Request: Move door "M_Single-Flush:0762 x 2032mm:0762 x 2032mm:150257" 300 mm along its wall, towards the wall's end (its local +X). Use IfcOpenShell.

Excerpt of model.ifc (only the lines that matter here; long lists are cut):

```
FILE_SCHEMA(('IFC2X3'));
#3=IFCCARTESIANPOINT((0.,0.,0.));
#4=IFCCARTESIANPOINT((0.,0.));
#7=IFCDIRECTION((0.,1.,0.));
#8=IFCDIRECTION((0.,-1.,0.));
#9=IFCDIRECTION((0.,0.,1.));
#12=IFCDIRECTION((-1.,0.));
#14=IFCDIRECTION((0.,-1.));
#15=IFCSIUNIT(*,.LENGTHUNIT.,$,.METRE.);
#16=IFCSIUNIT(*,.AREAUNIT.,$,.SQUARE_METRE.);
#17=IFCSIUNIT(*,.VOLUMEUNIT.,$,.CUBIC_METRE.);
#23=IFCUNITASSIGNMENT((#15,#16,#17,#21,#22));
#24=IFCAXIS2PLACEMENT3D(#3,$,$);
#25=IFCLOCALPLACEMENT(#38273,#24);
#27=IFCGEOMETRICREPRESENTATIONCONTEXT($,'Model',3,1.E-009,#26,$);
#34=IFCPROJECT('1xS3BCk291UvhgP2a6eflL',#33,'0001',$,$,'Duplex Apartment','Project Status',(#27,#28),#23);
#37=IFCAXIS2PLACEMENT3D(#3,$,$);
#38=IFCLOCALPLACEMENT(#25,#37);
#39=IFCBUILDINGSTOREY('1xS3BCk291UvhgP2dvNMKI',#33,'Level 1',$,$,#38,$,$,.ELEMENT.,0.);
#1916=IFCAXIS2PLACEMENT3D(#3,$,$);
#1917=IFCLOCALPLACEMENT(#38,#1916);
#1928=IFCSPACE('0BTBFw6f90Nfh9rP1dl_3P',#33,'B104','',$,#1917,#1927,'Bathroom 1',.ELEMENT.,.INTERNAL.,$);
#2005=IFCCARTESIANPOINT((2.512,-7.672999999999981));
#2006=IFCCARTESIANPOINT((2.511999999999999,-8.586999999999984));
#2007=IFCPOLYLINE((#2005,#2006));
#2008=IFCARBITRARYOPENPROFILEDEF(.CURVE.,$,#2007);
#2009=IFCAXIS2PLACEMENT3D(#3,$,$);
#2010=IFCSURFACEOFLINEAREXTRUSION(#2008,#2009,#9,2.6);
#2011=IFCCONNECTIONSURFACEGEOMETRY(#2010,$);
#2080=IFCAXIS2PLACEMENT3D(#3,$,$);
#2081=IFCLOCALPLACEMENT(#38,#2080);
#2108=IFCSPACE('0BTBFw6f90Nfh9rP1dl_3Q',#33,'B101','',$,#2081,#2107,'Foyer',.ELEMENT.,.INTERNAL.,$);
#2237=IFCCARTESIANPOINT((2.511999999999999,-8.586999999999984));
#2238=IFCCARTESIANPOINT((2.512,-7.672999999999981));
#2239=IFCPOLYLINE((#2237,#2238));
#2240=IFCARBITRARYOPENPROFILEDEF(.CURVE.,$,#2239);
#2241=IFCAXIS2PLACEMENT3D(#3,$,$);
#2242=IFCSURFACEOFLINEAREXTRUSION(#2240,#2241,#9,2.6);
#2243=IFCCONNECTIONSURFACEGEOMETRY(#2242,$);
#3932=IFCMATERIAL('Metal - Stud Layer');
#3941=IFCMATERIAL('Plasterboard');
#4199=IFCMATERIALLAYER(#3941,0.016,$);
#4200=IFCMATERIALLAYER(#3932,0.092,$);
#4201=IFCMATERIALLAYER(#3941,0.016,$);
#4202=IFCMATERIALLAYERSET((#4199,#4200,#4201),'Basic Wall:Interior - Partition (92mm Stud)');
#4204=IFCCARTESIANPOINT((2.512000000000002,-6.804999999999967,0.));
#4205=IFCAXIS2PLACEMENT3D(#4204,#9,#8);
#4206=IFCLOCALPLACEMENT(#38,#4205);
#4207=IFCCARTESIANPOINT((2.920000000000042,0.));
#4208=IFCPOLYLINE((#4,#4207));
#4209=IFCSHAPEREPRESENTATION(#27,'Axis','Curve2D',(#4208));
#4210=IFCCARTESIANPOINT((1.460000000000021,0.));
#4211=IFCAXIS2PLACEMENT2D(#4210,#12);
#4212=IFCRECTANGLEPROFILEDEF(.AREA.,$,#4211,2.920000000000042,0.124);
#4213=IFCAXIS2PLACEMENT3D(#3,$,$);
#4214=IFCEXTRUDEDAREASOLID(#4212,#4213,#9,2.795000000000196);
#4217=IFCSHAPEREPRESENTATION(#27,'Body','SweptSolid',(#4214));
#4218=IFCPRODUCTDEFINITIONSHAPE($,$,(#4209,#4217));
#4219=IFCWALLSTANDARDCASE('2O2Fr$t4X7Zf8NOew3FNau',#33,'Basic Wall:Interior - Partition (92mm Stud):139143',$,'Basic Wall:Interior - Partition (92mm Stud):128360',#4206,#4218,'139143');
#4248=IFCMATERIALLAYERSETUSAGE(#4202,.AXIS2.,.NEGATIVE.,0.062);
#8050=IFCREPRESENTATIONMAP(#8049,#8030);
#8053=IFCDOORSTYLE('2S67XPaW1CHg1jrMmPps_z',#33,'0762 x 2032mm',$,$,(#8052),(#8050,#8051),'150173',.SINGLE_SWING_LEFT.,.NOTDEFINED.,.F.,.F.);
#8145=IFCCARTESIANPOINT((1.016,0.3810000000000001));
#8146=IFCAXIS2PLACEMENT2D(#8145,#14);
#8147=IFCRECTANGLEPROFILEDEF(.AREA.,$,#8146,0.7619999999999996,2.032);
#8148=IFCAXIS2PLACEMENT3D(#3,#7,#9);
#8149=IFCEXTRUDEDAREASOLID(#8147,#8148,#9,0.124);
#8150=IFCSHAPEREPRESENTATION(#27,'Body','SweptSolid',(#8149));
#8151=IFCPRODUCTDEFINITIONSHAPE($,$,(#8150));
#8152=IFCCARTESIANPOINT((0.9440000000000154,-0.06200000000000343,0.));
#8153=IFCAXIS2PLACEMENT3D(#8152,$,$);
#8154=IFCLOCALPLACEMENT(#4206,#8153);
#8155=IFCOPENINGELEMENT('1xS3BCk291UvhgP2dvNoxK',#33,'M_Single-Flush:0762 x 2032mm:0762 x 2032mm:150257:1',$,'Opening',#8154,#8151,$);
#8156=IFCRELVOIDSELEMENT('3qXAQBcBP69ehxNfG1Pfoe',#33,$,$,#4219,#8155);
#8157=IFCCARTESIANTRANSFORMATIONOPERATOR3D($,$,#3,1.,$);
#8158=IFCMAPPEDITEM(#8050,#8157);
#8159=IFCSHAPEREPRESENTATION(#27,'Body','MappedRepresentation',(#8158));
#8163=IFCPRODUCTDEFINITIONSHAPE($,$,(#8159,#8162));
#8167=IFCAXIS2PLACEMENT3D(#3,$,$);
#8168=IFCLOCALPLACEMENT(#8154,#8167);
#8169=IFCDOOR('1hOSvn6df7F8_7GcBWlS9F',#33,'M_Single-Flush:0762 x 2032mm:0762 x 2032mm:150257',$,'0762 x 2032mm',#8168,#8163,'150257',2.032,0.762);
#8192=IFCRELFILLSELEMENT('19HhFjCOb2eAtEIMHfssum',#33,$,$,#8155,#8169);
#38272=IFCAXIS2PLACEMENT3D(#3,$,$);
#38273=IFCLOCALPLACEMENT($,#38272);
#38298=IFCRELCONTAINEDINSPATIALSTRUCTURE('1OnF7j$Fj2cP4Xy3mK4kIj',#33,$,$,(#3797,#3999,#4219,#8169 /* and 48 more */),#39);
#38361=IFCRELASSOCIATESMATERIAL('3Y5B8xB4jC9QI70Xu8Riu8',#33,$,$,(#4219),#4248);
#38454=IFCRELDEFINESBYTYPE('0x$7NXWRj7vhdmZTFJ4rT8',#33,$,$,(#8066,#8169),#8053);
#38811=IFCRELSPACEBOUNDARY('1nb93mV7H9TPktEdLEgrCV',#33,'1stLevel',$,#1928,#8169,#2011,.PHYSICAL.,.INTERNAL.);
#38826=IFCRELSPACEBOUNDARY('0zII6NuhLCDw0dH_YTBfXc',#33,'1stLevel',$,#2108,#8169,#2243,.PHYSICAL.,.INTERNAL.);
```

```python
import numpy as np
import ifcopenshell
import ifcopenshell.api.geometry
import ifcopenshell.util.placement
import ifcopenshell.util.unit

model = ifcopenshell.open("model.ifc")
unit_scale = ifcopenshell.util.unit.calculate_unit_scale(model)

door = model.by_guid("1hOSvn6df7F8_7GcBWlS9F")
opening = door.FillsVoids[0].RelatingOpeningElement
wall = opening.VoidsElements[0].RelatingBuildingElement

wall_matrix = ifcopenshell.util.placement.get_local_placement(wall.ObjectPlacement)
shift = wall_matrix[:3, 0] * 0.3 / unit_scale
before = ifcopenshell.util.placement.get_local_placement(door.ObjectPlacement)[:3, 3].copy()

# The door is placed relative to its opening, so it follows when the opening moves.
matrix = ifcopenshell.util.placement.get_local_placement(opening.ObjectPlacement)
matrix[:3, 3] += shift
ifcopenshell.api.geometry.edit_object_placement(
    model, product=opening, matrix=matrix, is_si=False, should_transform_children=True
)

# Space boundary surfaces are stored in each space's coordinates; move them too.
for rel in door.ProvidesBoundaries:
    if not rel.ConnectionGeometry:
        continue
    surface = rel.ConnectionGeometry.SurfaceOnRelatingElement
    space_matrix = ifcopenshell.util.placement.get_local_placement(rel.RelatingSpace.ObjectPlacement)
    point = np.array(surface.Position.Location.Coordinates) + space_matrix[:3, :3].T @ shift
    surface.Position = model.createIfcAxis2Placement3D(
        model.createIfcCartesianPoint(point.tolist()), surface.Position.Axis, surface.Position.RefDirection
    )

after = ifcopenshell.util.placement.get_local_placement(door.ObjectPlacement)[:3, 3]
print("door moved by", (after - before).round(3) + 0.0)

model.write("model_rev.ifc")
```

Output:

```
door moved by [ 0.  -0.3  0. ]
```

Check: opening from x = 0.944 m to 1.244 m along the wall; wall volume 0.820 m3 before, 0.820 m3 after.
